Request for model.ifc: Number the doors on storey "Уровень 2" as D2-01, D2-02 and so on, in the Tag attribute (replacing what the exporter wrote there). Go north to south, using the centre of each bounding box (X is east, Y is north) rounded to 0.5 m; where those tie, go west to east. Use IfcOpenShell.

First a look at what the model holds.

```python
import ifcopenshell
import ifcopenshell.util.element
import ifcopenshell.util.placement

model = ifcopenshell.open("model.ifc")
print(model.schema)
storey = next(s for s in model.by_type("IfcBuildingStorey") if s.Name == "Уровень 2")
doors = [e for e in ifcopenshell.util.element.get_decomposition(storey) if e.is_a("IfcDoor")]
for e in sorted(doors, key=lambda e: e.id()):
    origin = ifcopenshell.util.placement.get_local_placement(e.ObjectPlacement)[:3, 3]
    print(e.id(), e.Tag, e.Name, origin.round(2) + 0.0, sep=" | ")
```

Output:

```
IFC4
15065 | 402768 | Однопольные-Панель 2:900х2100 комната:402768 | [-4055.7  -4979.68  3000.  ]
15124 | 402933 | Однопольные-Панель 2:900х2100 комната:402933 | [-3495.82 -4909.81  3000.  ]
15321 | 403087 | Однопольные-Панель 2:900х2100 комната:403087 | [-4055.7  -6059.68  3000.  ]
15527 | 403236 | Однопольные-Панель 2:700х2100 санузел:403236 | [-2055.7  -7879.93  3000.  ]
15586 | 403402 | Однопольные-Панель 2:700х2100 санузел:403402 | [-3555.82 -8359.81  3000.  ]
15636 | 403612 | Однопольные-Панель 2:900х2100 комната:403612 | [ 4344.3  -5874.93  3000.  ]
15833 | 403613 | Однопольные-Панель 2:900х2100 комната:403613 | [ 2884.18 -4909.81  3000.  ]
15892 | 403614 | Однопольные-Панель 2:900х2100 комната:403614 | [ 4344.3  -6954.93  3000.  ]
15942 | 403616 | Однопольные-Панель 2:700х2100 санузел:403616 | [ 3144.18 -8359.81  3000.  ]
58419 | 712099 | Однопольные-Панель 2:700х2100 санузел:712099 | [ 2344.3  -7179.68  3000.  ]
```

```python
import ifcopenshell
import ifcopenshell.geom
import ifcopenshell.util.element
import ifcopenshell.util.shape

model = ifcopenshell.open("model.ifc")
settings = ifcopenshell.geom.settings()
settings.set("use-world-coords", True)


def centre(element):
    shape = ifcopenshell.geom.create_shape(settings, element)
    return ifcopenshell.util.shape.get_bbox_centroid(shape.geometry)


storey = next(s for s in model.by_type("IfcBuildingStorey") if s.Name == "Уровень 2")
doors = [e for e in ifcopenshell.util.element.get_decomposition(storey) if e.is_a("IfcDoor")]

# Insertion points can sit at a corner or the storey origin, so sort by the geometry (in metres).
centres = {e: centre(e) for e in doors}
doors.sort(key=lambda e: (-round(centres[e][1] / 0.5), centres[e][0]))

for i, e in enumerate(doors, start=1):
    number = f"D2-{i:02d}"
    e.Tag = number
    print(e.id(), number)

model.write("model_edited.ifc")
```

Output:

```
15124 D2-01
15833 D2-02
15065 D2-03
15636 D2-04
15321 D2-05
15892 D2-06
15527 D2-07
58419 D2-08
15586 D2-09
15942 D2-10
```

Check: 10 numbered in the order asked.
